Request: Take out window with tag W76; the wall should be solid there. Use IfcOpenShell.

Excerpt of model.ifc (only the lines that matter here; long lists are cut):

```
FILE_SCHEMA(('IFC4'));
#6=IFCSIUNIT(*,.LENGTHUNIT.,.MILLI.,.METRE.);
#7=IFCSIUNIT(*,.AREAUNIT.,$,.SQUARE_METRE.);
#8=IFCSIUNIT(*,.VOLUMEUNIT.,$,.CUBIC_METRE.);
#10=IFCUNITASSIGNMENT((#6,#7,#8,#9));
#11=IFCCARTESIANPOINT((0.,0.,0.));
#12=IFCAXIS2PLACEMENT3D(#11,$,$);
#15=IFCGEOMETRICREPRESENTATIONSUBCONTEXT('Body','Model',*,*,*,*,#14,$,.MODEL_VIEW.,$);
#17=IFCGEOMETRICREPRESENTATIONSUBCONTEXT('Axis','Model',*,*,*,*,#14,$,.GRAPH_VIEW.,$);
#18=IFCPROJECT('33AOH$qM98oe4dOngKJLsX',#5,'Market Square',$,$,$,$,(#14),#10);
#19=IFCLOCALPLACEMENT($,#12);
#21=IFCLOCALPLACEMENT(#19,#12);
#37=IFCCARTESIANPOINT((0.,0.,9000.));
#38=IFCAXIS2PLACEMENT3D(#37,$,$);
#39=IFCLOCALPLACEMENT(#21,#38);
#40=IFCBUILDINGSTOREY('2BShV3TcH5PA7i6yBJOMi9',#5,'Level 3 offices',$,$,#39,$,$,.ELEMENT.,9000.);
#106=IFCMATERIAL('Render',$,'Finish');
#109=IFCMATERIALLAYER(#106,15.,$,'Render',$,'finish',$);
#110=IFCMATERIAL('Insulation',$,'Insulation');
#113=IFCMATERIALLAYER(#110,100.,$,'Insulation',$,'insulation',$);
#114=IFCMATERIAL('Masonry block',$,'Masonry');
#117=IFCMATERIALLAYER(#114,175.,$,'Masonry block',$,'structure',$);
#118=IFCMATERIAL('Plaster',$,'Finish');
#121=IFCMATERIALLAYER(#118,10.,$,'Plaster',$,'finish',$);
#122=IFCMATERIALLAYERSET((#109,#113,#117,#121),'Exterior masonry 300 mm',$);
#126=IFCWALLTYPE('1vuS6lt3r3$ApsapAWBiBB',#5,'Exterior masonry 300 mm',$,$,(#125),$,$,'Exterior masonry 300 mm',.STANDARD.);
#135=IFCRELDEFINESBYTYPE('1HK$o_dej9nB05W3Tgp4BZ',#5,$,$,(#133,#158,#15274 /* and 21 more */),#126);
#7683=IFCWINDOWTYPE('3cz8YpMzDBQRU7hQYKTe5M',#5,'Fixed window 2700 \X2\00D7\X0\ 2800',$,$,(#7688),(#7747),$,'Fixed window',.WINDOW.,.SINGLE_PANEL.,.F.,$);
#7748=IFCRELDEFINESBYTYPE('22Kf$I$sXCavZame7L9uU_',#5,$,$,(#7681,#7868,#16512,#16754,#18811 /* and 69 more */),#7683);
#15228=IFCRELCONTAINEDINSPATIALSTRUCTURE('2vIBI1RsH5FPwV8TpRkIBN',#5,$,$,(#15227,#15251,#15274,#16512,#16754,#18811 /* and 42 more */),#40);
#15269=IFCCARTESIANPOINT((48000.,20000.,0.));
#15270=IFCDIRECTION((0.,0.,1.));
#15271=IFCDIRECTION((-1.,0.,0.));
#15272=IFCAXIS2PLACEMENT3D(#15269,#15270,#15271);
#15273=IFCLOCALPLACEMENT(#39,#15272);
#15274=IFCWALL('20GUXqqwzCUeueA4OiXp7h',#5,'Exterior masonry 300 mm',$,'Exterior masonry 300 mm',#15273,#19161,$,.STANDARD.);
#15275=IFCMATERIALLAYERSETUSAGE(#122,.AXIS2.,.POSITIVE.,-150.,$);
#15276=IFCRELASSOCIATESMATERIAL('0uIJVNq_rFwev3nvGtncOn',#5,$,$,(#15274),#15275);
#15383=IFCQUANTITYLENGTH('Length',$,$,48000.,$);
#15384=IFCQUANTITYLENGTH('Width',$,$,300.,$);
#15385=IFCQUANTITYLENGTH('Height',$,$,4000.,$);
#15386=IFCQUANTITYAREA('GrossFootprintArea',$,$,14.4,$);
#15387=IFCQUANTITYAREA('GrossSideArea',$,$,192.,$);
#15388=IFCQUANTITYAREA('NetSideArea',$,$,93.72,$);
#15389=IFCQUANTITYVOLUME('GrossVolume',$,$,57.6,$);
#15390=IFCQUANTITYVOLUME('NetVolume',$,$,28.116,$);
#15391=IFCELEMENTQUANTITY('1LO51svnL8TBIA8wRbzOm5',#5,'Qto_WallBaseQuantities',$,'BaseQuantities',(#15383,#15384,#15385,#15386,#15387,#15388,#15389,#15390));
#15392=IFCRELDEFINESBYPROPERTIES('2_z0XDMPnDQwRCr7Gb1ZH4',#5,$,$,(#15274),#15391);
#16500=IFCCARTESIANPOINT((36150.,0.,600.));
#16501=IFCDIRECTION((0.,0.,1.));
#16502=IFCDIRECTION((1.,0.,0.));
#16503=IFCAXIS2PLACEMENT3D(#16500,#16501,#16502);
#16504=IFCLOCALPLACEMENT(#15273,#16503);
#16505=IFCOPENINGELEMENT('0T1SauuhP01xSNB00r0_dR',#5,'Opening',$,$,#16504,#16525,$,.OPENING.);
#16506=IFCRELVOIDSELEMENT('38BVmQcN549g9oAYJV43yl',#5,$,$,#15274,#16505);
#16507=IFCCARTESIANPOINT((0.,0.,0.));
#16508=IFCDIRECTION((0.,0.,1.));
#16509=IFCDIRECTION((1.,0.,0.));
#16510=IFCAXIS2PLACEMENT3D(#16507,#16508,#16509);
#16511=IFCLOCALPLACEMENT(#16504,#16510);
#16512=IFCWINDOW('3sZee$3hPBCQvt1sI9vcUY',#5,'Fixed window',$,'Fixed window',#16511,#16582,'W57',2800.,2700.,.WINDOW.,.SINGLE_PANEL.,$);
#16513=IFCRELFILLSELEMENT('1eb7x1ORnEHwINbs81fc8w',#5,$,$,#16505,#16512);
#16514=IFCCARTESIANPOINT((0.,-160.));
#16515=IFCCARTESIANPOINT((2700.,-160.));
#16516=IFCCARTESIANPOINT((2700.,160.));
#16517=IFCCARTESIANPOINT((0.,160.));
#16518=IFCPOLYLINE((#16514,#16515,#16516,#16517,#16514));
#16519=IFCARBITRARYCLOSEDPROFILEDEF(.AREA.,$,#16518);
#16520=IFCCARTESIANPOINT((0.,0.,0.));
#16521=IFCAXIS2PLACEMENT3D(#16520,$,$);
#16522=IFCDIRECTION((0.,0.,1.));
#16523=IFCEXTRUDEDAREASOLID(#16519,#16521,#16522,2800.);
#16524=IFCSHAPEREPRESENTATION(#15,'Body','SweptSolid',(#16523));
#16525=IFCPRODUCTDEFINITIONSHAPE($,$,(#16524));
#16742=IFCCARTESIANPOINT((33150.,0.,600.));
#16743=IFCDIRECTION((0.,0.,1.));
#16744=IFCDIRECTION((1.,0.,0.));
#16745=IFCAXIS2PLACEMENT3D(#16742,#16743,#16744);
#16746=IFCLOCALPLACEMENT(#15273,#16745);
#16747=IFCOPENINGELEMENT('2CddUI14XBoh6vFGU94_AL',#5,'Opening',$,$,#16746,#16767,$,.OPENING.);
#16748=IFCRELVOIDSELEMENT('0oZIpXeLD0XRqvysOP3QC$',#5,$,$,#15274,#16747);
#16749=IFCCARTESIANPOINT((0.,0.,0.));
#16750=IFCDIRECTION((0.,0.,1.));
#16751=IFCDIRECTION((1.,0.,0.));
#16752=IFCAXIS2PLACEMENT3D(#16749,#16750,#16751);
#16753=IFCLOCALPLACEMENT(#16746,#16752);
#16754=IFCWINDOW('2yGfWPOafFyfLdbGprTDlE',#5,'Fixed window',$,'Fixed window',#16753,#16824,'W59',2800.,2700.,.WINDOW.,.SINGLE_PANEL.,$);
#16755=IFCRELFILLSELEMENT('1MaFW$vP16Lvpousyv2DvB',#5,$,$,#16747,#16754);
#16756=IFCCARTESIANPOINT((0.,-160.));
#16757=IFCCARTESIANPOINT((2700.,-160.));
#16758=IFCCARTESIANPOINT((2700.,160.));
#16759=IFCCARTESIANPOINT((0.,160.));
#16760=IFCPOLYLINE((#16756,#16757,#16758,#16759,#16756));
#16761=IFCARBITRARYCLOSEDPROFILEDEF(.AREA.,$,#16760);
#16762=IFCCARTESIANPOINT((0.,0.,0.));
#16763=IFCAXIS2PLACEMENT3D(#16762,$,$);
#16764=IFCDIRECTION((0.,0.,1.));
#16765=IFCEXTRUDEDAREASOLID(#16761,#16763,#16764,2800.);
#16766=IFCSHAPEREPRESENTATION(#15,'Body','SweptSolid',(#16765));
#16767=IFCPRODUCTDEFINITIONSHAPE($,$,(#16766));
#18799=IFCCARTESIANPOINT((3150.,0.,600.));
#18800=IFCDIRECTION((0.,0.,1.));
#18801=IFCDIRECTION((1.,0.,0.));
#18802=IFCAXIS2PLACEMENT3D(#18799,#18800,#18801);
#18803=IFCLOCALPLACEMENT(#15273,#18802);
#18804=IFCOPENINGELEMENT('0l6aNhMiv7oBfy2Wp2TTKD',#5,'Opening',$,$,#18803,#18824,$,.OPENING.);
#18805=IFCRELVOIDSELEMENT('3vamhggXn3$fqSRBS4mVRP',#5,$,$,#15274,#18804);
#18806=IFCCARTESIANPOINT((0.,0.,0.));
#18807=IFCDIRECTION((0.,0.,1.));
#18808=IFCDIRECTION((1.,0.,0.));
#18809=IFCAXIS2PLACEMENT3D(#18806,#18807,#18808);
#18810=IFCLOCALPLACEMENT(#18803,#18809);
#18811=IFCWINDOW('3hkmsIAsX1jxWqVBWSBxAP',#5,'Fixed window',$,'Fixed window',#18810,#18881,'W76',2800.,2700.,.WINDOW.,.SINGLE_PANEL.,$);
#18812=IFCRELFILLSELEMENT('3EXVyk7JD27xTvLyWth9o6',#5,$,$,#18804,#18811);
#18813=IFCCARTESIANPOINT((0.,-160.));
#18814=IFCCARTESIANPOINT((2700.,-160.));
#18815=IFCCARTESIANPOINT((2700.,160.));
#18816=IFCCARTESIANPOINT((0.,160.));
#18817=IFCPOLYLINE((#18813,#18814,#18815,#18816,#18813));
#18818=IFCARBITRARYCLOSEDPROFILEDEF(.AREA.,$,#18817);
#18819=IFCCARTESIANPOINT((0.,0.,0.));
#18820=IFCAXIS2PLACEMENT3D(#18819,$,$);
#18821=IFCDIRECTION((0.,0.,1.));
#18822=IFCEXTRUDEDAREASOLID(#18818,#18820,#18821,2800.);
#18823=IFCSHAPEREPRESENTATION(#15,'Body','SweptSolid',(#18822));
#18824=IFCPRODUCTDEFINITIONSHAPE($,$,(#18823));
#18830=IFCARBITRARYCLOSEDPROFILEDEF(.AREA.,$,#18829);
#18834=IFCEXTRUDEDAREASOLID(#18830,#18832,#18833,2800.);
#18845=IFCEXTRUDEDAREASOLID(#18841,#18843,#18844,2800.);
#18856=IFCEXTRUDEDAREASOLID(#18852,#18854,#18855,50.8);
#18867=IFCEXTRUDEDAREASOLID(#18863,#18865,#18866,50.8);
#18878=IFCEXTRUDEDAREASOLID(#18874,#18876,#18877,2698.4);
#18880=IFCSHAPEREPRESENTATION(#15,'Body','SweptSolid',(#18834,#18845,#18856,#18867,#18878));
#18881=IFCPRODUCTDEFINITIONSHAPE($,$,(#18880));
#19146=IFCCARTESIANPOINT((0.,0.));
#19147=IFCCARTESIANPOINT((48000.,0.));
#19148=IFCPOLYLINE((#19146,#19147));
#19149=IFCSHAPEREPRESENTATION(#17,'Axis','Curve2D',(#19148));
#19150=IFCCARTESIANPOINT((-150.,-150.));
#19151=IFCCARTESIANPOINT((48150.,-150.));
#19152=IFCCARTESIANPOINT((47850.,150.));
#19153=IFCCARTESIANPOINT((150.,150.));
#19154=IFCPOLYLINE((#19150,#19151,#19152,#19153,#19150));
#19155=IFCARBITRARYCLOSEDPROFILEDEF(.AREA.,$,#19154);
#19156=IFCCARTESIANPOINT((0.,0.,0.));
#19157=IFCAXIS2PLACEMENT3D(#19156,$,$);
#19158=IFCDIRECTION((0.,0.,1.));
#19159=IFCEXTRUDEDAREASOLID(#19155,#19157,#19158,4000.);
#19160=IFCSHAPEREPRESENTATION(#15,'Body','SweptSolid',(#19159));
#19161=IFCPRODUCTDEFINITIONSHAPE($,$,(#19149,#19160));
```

```python
import ifcopenshell
import ifcopenshell.api.feature
import ifcopenshell.api.pset
import ifcopenshell.api.root
import ifcopenshell.geom
import ifcopenshell.util.element
import ifcopenshell.util.shape
import ifcopenshell.util.unit

model = ifcopenshell.open("model.ifc")
area_scale = ifcopenshell.util.unit.calculate_unit_scale(model, "AREAUNIT")
volume_scale = ifcopenshell.util.unit.calculate_unit_scale(model, "VOLUMEUNIT")
settings = ifcopenshell.geom.settings()


def volume(element):
    """Net volume in cubic metres, openings subtracted."""
    shape = ifcopenshell.geom.create_shape(settings, element)
    return ifcopenshell.util.shape.get_volume(shape.geometry)


window = model.by_guid("3hkmsIAsX1jxWqVBWSBxAP")
opening = window.FillsVoids[0].RelatingOpeningElement
wall = opening.VoidsElements[0].RelatingBuildingElement
before = volume(wall)

ifcopenshell.api.root.remove_product(model, product=window)
ifcopenshell.api.feature.remove_feature(model, feature=opening)

after = volume(wall)
thickness = 0.3  # wall thickness in metres

# Update the wall's stored quantities.
qto = model.by_id(ifcopenshell.util.element.get_pset(wall, "Qto_WallBaseQuantities", should_inherit=False)["id"])
ifcopenshell.api.pset.edit_qto(model, qto=qto, properties={
    "NetSideArea": after / thickness / area_scale,
    "NetVolume": after / volume_scale,
})

print(f"wall volume {before:.3f} -> {after:.3f} m3")

model.write("model_rev.ifc")
```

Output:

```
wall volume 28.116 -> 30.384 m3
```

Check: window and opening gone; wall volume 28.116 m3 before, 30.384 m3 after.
